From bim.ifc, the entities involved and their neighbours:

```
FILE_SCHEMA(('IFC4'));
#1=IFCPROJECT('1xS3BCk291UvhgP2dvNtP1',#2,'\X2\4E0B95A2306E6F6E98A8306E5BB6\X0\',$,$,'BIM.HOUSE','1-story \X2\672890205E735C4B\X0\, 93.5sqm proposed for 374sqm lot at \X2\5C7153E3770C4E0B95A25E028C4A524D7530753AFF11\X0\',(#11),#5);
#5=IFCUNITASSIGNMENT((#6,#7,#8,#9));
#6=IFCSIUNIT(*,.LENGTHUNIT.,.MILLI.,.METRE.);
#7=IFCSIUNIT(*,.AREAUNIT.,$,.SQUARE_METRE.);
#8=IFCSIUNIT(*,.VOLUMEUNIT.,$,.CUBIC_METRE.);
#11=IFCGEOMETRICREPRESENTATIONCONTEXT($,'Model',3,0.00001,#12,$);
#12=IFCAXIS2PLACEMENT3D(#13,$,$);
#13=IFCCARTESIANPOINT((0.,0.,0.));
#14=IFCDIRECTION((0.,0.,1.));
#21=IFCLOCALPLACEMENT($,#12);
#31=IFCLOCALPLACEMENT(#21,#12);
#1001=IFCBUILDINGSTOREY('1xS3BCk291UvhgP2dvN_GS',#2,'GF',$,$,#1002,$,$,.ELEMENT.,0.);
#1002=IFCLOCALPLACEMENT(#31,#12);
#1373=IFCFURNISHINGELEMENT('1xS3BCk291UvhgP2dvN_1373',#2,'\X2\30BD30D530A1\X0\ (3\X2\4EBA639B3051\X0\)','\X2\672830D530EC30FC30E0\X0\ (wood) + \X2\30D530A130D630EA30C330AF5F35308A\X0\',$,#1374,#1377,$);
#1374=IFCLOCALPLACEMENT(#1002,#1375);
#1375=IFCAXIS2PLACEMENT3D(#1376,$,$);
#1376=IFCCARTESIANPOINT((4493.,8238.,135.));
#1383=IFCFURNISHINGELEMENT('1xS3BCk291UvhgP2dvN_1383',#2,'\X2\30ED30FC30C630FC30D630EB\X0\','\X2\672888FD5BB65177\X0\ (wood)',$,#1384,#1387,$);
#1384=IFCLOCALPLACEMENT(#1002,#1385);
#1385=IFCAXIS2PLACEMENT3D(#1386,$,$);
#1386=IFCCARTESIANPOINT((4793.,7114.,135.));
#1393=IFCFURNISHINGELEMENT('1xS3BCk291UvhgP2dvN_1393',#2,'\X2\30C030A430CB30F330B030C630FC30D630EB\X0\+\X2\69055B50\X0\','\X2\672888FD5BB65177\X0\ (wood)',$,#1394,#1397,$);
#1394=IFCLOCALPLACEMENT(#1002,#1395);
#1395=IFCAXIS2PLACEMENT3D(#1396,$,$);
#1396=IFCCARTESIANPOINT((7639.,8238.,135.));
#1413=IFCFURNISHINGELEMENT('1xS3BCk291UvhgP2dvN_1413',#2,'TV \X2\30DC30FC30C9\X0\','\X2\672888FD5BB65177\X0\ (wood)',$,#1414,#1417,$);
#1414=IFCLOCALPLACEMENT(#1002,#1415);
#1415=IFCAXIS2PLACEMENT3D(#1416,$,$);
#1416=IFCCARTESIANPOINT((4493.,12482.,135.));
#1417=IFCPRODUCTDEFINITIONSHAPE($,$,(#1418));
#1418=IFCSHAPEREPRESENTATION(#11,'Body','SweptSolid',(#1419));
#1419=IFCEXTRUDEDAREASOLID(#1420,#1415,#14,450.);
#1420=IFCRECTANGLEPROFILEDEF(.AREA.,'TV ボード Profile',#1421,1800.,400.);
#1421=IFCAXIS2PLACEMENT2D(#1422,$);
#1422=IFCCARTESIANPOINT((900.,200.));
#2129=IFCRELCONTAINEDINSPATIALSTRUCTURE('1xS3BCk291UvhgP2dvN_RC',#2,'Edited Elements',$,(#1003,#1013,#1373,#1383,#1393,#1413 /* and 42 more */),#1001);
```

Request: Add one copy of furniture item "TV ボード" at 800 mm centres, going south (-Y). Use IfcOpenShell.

```python
import numpy as np
import ifcopenshell
import ifcopenshell.api.geometry
import ifcopenshell.api.root
import ifcopenshell.util.element
import ifcopenshell.util.placement

model = ifcopenshell.open("bim.ifc")


def reuse_history(source, copy):
    """copy_class also copies each property set's owner history, people and application; keep the originals."""
    for rel in copy.IsDefinedBy:
        if rel.is_a("IfcRelDefinesByProperties") and (history := rel.RelatingPropertyDefinition.OwnerHistory):
            rel.RelatingPropertyDefinition.OwnerHistory = source.OwnerHistory
            ifcopenshell.util.element.remove_deep2(model, history)


source = model.by_guid("1xS3BCk291UvhgP2dvN_1413")
base = ifcopenshell.util.placement.get_local_placement(source.ObjectPlacement)
step = np.array([0.0, -1.0, 0.0]) * 800.0

for i in range(1, 2):
    copy = ifcopenshell.api.root.copy_class(model, product=source)
    copy.Representation = ifcopenshell.util.element.copy_deep(
        model, source.Representation, exclude=["IfcGeometricRepresentationContext", "IfcRepresentationMap"]
    )
    reuse_history(source, copy)
    matrix = base.copy()
    matrix[:3, 3] += i * step
    print("added at", matrix[:3, 3].round(3) + 0.0)
    ifcopenshell.api.geometry.edit_object_placement(model, product=copy, matrix=matrix, is_si=False)

model.write("bim_rev.ifc")
```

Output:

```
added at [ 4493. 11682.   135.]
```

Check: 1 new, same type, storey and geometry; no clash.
